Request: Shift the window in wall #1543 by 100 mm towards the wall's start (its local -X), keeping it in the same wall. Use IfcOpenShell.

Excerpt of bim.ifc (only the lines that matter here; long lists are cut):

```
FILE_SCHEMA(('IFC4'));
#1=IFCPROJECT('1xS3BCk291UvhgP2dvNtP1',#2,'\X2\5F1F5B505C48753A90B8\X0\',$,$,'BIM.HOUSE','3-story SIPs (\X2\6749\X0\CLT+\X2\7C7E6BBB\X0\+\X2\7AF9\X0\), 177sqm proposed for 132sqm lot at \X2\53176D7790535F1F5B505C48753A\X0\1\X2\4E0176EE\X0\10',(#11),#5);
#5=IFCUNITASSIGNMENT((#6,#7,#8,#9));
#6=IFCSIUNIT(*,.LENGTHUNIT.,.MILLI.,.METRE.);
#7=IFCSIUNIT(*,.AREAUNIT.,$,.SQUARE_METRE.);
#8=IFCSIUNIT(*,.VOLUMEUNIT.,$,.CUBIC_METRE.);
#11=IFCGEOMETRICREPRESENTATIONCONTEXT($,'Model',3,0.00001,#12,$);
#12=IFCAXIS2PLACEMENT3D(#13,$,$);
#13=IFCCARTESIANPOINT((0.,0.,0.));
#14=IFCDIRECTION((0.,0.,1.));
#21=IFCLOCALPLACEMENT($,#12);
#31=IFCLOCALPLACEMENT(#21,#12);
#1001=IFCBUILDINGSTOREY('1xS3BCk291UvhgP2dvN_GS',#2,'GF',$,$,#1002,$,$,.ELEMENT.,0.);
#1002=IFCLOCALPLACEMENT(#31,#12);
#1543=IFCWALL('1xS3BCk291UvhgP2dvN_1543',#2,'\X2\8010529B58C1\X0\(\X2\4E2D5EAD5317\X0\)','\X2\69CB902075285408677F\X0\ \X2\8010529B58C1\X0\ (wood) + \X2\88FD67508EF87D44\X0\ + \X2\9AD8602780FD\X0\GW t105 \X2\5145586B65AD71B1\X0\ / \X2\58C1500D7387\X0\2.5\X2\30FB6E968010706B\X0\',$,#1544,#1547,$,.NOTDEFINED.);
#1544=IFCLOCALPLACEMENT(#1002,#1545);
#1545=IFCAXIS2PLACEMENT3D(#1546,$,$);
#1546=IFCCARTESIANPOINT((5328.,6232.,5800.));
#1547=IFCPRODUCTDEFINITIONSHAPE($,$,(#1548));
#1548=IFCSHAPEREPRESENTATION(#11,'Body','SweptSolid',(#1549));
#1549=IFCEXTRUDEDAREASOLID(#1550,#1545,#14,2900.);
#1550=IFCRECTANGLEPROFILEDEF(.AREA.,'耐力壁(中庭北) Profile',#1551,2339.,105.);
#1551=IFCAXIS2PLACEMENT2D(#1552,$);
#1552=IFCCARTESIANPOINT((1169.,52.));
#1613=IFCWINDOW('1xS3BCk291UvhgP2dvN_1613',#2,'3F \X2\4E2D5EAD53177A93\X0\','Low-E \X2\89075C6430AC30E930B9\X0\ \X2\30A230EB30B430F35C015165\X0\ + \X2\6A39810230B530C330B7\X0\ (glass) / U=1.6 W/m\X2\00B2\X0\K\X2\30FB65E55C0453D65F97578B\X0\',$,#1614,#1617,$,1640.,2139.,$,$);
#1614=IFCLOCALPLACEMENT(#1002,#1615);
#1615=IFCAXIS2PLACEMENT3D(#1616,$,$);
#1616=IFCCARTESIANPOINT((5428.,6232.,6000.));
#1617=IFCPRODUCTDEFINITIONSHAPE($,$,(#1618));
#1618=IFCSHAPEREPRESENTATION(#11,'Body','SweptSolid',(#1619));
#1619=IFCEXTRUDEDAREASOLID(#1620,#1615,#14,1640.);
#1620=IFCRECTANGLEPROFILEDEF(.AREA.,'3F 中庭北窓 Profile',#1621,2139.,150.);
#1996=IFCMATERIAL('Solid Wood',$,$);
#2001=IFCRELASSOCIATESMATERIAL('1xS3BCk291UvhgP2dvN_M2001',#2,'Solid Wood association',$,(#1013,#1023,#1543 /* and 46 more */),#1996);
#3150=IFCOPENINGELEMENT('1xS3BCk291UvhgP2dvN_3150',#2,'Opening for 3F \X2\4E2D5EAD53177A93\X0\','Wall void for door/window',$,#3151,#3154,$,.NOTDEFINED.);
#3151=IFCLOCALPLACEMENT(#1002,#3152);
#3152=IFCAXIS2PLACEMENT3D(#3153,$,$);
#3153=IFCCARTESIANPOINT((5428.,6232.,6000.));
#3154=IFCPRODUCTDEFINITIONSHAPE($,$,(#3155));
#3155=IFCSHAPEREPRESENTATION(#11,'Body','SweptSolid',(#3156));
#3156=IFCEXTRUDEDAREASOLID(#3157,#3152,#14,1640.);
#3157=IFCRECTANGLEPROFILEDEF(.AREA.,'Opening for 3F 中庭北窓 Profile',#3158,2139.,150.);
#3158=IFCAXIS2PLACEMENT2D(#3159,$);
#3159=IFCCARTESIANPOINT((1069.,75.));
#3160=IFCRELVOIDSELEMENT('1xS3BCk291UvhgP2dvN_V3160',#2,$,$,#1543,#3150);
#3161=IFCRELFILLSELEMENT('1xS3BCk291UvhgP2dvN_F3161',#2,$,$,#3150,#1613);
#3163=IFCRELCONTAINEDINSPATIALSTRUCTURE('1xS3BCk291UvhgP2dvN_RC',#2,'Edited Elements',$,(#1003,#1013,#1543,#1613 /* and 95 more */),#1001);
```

```python
import ifcopenshell
import ifcopenshell.api.geometry
import ifcopenshell.util.placement

model = ifcopenshell.open("bim.ifc")

window = model.by_guid("1xS3BCk291UvhgP2dvN_1613")
opening = window.FillsVoids[0].RelatingOpeningElement
wall = opening.VoidsElements[0].RelatingBuildingElement

wall_matrix = ifcopenshell.util.placement.get_local_placement(wall.ObjectPlacement)
shift = wall_matrix[:3, 0] * -100.0
before = ifcopenshell.util.placement.get_local_placement(window.ObjectPlacement)[:3, 3].copy()

# The window is not placed relative to its opening, so move both.
for product in (opening, window):
    matrix = ifcopenshell.util.placement.get_local_placement(product.ObjectPlacement)
    matrix[:3, 3] += shift
    ifcopenshell.api.geometry.edit_object_placement(model, product=product, matrix=matrix, is_si=False)

after = ifcopenshell.util.placement.get_local_placement(window.ObjectPlacement)[:3, 3]
print("window moved by", (after - before).round(3) + 0.0)

model.write("bim_v2.ifc")
```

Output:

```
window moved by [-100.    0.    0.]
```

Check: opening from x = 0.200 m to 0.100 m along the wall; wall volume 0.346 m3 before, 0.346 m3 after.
